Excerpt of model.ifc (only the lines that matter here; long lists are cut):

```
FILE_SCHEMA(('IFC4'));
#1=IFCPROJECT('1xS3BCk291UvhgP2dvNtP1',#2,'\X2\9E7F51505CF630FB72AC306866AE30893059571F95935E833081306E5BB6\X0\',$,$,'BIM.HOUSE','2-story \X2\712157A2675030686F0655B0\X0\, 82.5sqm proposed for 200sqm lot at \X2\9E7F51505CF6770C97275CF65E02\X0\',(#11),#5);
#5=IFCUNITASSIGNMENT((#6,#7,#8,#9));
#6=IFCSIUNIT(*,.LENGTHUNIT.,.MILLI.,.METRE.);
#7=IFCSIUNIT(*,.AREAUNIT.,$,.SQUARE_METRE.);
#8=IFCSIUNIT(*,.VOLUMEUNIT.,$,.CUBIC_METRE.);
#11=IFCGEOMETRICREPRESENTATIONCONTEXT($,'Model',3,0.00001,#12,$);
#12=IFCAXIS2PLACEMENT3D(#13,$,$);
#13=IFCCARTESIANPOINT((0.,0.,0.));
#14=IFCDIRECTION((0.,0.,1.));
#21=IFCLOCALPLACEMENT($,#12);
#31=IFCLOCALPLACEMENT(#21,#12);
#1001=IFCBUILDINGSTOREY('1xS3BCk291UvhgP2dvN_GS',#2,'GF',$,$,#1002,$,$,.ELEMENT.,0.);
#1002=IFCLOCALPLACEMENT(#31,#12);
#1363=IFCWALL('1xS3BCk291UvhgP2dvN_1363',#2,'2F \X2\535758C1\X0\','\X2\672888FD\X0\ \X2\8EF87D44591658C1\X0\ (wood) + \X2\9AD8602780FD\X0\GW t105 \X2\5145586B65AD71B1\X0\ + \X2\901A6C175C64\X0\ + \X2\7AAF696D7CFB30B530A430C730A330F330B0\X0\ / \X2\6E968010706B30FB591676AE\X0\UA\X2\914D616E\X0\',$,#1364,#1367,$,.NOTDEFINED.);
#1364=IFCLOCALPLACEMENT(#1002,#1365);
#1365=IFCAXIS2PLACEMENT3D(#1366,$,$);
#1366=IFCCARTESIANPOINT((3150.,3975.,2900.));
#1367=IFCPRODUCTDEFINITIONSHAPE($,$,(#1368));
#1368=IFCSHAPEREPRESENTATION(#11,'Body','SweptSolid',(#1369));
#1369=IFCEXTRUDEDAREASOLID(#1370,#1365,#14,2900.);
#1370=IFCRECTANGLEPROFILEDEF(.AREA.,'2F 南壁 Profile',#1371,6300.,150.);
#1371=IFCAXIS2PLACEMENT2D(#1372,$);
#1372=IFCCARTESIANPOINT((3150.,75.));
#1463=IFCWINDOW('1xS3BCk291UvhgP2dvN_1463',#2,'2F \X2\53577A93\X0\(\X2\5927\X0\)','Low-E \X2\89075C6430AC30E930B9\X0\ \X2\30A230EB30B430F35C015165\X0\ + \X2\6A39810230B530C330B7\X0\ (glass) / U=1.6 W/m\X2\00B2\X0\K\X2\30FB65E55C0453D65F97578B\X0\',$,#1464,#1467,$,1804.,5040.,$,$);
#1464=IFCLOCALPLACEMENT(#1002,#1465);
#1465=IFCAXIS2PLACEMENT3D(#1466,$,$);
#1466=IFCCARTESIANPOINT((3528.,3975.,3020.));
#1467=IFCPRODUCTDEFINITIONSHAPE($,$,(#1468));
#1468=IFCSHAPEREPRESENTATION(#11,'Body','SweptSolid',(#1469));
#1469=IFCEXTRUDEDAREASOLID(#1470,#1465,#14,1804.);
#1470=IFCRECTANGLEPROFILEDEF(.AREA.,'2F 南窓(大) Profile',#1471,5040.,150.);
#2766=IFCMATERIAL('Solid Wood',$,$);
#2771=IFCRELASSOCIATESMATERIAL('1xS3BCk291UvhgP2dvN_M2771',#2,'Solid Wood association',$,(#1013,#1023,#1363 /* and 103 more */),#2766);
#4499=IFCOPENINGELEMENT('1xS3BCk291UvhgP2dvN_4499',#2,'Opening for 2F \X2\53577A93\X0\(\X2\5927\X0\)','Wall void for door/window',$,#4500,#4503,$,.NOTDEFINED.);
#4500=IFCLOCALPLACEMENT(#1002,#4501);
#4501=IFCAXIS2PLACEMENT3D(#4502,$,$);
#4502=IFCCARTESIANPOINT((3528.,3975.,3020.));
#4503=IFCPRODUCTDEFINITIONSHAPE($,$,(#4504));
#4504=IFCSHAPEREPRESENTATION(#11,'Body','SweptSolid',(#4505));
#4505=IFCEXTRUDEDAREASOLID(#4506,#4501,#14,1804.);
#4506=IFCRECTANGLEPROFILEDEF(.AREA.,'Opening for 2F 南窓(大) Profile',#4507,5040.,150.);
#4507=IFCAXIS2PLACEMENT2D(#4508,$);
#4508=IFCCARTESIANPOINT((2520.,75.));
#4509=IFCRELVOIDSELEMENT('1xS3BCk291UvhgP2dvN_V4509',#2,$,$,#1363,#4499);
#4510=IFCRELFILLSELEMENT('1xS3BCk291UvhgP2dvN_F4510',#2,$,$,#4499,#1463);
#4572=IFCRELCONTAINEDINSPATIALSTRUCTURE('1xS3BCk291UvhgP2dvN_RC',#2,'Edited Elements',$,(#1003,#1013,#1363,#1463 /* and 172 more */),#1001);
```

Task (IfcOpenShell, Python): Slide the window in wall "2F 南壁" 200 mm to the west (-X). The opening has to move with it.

```python
import ifcopenshell
import ifcopenshell.api.geometry
import ifcopenshell.util.placement
import ifcopenshell.util.unit

model = ifcopenshell.open("model.ifc")
unit_scale = ifcopenshell.util.unit.calculate_unit_scale(model)

window = model.by_guid("1xS3BCk291UvhgP2dvN_1463")
opening = window.FillsVoids[0].RelatingOpeningElement
wall = opening.VoidsElements[0].RelatingBuildingElement

wall_matrix = ifcopenshell.util.placement.get_local_placement(wall.ObjectPlacement)
shift = wall_matrix[:3, 0] * -0.2 / unit_scale
before = ifcopenshell.util.placement.get_local_placement(window.ObjectPlacement)[:3, 3].copy()

# The window is not placed relative to its opening, so move both.
for product in (opening, window):
    matrix = ifcopenshell.util.placement.get_local_placement(product.ObjectPlacement)
    matrix[:3, 3] += shift
    ifcopenshell.api.geometry.edit_object_placement(model, product=product, matrix=matrix, is_si=False)

after = ifcopenshell.util.placement.get_local_placement(window.ObjectPlacement)[:3, 3]
print("window moved by", (after - before).round(3) + 0.0)

model.write("model_v2.ifc")
```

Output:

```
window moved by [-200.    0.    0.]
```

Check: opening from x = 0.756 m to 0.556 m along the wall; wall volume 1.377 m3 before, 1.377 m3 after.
